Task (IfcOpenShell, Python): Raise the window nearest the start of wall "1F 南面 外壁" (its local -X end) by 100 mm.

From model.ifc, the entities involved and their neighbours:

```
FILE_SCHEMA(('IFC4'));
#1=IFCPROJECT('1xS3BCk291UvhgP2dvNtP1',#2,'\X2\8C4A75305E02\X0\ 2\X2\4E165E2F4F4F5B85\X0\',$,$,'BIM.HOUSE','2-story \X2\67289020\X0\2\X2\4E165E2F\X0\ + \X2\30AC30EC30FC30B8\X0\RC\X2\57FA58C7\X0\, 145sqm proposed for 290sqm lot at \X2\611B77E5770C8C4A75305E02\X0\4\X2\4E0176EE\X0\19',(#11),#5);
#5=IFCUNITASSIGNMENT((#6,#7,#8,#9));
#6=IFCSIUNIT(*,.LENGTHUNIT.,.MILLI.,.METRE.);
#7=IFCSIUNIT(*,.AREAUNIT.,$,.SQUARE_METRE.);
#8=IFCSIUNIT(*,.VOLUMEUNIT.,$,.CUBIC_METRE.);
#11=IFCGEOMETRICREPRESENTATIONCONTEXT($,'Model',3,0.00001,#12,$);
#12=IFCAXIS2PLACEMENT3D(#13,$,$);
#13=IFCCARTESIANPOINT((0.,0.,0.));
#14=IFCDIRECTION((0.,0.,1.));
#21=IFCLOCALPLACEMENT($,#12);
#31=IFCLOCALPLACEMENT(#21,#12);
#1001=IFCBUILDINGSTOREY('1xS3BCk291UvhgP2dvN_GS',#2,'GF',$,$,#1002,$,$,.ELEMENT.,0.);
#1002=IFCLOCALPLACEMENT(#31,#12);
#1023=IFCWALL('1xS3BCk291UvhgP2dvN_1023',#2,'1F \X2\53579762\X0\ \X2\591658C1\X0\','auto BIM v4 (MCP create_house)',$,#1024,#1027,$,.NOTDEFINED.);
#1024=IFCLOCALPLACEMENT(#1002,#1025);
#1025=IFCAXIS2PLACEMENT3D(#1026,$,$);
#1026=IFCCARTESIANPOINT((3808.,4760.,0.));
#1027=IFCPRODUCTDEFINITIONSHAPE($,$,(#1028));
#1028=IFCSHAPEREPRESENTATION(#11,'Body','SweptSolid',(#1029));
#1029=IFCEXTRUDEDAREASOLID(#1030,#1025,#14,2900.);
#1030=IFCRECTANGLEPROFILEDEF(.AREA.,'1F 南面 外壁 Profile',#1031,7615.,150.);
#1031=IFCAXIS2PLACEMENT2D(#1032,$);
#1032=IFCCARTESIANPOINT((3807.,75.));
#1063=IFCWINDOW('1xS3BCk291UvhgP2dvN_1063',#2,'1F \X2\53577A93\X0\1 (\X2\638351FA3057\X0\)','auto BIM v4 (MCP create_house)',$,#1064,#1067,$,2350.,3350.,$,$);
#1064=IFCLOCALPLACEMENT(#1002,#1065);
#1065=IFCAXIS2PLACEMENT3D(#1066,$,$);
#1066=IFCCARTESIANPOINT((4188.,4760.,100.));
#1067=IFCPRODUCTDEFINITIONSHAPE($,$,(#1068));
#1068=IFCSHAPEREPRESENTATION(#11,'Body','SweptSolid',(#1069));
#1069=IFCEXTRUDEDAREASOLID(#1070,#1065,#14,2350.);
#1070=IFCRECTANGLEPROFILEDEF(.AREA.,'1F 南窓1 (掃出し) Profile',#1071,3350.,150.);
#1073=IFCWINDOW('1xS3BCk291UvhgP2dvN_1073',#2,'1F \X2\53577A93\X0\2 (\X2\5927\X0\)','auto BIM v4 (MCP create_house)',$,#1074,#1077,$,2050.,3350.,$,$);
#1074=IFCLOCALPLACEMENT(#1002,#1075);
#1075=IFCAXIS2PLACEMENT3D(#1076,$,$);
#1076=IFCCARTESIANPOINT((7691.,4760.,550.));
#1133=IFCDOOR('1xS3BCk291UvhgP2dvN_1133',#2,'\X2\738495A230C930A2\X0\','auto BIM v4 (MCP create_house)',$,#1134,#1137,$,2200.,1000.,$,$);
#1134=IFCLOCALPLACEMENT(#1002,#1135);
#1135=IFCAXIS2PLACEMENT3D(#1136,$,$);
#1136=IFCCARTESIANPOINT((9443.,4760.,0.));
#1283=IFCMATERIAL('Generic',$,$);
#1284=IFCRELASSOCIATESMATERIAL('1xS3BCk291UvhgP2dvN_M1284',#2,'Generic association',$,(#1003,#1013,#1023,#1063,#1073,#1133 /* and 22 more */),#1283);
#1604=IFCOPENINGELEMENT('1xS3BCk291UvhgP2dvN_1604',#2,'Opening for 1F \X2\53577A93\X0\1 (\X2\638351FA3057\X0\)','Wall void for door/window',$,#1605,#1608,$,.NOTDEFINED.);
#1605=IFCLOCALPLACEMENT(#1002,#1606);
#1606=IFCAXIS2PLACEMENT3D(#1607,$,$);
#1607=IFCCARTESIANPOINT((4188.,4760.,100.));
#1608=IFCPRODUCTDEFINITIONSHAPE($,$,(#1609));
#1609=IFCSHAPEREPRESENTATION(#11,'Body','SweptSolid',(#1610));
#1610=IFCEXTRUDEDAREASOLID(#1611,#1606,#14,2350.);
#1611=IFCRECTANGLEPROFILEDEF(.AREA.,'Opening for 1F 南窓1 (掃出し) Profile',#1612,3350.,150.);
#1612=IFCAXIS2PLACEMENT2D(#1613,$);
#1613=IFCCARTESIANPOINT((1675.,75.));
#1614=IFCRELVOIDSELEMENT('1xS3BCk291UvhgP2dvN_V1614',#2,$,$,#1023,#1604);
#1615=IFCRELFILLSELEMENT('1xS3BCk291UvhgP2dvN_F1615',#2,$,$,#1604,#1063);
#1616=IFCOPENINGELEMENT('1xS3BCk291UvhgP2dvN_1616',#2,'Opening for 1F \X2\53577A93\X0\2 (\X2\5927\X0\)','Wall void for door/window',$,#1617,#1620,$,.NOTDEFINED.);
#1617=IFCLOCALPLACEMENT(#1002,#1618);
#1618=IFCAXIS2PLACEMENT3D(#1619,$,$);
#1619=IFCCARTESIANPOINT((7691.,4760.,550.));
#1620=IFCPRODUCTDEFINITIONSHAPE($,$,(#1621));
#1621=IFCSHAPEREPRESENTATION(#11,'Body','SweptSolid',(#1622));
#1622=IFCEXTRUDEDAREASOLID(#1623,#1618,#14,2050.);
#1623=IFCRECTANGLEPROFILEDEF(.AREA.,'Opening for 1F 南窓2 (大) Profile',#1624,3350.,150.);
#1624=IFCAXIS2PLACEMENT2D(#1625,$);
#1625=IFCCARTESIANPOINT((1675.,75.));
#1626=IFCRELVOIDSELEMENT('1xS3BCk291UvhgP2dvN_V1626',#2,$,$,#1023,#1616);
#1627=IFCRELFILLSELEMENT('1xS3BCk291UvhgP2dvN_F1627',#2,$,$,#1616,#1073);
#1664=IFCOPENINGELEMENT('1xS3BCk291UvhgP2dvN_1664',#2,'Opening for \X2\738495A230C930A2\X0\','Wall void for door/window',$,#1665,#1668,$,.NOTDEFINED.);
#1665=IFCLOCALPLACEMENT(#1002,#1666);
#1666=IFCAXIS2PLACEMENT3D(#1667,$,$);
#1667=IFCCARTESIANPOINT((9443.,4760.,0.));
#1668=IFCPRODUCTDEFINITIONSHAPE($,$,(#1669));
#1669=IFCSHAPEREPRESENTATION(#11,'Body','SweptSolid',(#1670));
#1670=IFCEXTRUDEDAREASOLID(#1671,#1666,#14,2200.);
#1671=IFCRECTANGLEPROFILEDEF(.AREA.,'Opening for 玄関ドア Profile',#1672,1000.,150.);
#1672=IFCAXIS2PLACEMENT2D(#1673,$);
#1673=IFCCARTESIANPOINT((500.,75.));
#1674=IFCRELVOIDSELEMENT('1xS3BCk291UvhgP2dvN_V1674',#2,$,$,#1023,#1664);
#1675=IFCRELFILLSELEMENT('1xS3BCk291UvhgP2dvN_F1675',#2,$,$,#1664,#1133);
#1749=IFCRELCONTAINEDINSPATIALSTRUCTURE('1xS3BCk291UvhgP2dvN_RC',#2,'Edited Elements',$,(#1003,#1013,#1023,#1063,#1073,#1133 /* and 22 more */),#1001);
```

```python
import numpy as np
import ifcopenshell
import ifcopenshell.api.geometry
import ifcopenshell.util.placement
import ifcopenshell.util.unit

model = ifcopenshell.open("model.ifc")
unit_scale = ifcopenshell.util.unit.calculate_unit_scale(model)

window = model.by_guid("1xS3BCk291UvhgP2dvN_1063")
opening = window.FillsVoids[0].RelatingOpeningElement
dz = 0.1 / unit_scale

shift = np.array([0.0, 0.0, dz])
# The window is not placed relative to its opening, so move both.
for product in (opening, window):
    matrix = ifcopenshell.util.placement.get_local_placement(product.ObjectPlacement)
    matrix[:3, 3] += shift
    ifcopenshell.api.geometry.edit_object_placement(model, product=product, matrix=matrix, is_si=False)

print(f"moved by {dz * unit_scale:+.3f} m")

model.write("model_edited.ifc")
```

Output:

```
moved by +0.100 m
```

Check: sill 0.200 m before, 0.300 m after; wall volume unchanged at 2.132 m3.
